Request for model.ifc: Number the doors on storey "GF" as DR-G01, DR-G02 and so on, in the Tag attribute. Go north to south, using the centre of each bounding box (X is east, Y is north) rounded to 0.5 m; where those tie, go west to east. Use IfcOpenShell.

First a look at what the model holds.

```python
import ifcopenshell
import ifcopenshell.util.element
import ifcopenshell.util.placement

model = ifcopenshell.open("model.ifc")
print(model.schema)
storey = next(s for s in model.by_type("IfcBuildingStorey") if s.Name == "GF")
doors = [e for e in ifcopenshell.util.element.get_decomposition(storey) if e.is_a("IfcDoor")]
for e in sorted(doors, key=lambda e: e.id()):
    origin = ifcopenshell.util.placement.get_local_placement(e.ObjectPlacement)[:3, 3]
    print(e.id(), e.Tag, e.Name, origin.round(2) + 0.0, sep=" | ")
```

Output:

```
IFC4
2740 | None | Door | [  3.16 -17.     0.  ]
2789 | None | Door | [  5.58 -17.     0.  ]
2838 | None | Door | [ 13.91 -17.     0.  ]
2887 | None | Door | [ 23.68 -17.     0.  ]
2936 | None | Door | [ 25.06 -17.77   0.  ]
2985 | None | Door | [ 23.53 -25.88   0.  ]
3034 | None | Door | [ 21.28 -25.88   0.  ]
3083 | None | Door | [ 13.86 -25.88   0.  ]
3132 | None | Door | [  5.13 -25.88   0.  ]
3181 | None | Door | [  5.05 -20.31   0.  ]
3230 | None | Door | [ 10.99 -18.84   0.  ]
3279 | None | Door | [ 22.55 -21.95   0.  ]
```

```python
import ifcopenshell
import ifcopenshell.geom
import ifcopenshell.util.element
import ifcopenshell.util.shape

model = ifcopenshell.open("model.ifc")
settings = ifcopenshell.geom.settings()
settings.set("use-world-coords", True)


def centre(element):
    shape = ifcopenshell.geom.create_shape(settings, element)
    return ifcopenshell.util.shape.get_bbox_centroid(shape.geometry)


storey = next(s for s in model.by_type("IfcBuildingStorey") if s.Name == "GF")
doors = [e for e in ifcopenshell.util.element.get_decomposition(storey) if e.is_a("IfcDoor")]

# Insertion points can sit at a corner or the storey origin, so sort by the geometry (in metres).
centres = {e: centre(e) for e in doors}
doors.sort(key=lambda e: (-round(centres[e][1] / 0.5), centres[e][0]))

for i, e in enumerate(doors, start=1):
    number = f"DR-G{i:02d}"
    e.Tag = number
    print(e.id(), number)

model.write("model_v2.ifc")
```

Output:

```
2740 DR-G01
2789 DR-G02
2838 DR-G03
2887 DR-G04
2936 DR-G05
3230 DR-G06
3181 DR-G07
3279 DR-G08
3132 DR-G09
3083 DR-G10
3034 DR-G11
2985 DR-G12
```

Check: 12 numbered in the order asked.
